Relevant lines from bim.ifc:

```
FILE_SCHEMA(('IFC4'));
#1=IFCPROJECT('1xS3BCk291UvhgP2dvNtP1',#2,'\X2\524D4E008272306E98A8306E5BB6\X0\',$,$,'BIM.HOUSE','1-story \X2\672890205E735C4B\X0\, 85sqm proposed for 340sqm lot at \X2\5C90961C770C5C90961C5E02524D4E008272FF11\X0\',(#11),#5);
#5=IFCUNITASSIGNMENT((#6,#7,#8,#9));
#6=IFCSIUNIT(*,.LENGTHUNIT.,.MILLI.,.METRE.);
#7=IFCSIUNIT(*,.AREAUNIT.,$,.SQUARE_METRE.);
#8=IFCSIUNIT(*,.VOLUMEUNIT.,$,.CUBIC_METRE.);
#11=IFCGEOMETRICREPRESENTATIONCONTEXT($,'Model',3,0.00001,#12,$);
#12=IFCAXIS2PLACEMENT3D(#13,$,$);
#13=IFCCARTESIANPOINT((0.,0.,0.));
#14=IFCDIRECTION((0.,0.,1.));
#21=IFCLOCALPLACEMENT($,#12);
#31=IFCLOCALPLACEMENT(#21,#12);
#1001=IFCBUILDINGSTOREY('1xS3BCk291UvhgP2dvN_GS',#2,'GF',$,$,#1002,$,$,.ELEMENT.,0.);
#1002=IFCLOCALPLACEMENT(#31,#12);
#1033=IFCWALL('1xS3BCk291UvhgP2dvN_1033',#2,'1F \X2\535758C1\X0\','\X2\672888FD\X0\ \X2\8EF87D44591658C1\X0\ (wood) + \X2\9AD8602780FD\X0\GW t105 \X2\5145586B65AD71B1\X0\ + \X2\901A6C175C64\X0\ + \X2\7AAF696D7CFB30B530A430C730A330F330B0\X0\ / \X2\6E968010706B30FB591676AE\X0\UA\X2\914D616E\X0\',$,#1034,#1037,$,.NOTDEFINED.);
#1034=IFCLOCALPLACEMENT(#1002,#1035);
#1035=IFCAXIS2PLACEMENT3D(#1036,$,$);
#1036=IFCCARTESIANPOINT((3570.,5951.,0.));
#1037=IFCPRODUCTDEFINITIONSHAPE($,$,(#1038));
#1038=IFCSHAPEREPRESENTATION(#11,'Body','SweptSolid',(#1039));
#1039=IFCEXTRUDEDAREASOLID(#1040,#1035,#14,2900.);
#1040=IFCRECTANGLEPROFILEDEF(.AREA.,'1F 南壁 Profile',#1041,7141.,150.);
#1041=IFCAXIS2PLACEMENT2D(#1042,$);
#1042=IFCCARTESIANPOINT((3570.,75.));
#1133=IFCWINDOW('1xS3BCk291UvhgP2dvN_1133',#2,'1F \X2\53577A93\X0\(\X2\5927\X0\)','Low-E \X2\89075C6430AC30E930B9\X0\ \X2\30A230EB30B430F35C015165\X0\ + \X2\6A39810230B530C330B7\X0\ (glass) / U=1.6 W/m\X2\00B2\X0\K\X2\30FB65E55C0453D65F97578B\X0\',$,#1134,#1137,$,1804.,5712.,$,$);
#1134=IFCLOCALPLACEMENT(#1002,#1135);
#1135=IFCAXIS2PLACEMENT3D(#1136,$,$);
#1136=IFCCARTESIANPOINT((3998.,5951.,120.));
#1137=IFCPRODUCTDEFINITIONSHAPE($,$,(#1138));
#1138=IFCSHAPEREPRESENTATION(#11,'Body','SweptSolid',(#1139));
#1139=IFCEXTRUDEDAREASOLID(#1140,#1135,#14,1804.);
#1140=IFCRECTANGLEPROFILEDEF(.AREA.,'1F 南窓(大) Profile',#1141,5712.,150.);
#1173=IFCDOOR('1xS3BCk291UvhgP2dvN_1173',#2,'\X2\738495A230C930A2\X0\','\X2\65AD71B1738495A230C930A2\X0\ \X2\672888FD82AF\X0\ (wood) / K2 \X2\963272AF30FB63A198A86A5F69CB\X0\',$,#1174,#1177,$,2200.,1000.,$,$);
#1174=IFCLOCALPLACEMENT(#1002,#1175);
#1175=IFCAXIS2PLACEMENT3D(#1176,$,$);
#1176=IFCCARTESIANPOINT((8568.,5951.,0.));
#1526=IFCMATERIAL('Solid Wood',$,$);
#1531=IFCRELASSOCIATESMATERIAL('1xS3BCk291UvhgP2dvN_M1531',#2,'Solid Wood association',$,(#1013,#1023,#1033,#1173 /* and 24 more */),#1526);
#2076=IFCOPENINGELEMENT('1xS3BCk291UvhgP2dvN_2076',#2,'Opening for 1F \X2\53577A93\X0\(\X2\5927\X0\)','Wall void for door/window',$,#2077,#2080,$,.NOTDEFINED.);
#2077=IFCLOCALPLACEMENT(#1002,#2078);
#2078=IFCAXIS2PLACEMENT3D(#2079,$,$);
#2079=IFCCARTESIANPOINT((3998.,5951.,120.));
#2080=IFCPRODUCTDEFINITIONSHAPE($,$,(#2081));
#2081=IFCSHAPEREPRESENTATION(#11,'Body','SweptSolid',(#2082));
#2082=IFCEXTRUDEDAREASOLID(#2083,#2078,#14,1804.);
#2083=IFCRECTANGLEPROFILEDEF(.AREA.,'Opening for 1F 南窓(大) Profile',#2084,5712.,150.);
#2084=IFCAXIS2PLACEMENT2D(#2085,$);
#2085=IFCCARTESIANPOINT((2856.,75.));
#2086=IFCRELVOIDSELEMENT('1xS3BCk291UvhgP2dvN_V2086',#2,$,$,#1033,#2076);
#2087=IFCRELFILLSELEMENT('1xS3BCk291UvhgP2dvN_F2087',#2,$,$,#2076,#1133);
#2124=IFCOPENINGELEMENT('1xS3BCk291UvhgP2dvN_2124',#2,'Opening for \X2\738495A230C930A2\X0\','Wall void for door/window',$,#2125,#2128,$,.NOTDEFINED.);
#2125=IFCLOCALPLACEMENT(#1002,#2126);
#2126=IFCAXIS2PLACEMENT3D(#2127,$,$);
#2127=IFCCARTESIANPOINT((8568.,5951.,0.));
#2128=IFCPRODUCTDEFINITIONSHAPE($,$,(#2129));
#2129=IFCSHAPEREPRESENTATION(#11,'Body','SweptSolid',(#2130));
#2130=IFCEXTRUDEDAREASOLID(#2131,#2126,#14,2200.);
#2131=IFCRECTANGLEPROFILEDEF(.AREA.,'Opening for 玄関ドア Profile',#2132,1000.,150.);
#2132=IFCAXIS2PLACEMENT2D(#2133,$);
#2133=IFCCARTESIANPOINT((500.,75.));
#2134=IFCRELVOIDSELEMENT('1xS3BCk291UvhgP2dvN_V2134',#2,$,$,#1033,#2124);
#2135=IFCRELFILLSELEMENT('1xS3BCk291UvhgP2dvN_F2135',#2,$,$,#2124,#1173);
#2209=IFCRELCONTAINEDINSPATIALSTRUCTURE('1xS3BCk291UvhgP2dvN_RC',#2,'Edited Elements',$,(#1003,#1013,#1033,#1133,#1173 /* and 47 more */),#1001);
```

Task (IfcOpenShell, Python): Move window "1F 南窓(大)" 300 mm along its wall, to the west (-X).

```python
import ifcopenshell
import ifcopenshell.api.geometry
import ifcopenshell.util.placement

model = ifcopenshell.open("bim.ifc")

window = model.by_guid("1xS3BCk291UvhgP2dvN_1133")
opening = window.FillsVoids[0].RelatingOpeningElement
wall = opening.VoidsElements[0].RelatingBuildingElement

wall_matrix = ifcopenshell.util.placement.get_local_placement(wall.ObjectPlacement)
shift = wall_matrix[:3, 0] * -300.0
before = ifcopenshell.util.placement.get_local_placement(window.ObjectPlacement)[:3, 3].copy()

# The window is not placed relative to its opening, so move both.
for product in (opening, window):
    matrix = ifcopenshell.util.placement.get_local_placement(product.ObjectPlacement)
    matrix[:3, 3] += shift
    ifcopenshell.api.geometry.edit_object_placement(model, product=product, matrix=matrix, is_si=False)

after = ifcopenshell.util.placement.get_local_placement(window.ObjectPlacement)[:3, 3]
print("window moved by", (after - before).round(3) + 0.0)

model.write("bim_v2.ifc")
```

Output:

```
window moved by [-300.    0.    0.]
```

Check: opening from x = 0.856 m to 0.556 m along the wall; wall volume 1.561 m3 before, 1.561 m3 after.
